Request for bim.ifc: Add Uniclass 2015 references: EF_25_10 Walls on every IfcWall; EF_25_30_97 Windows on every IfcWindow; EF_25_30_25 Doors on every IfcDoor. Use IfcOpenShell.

First a look at what the model holds.

```python
import ifcopenshell

model = ifcopenshell.open("bim.ifc")
print(model.schema)
print("classifications:", [c.Name for c in model.by_type("IfcClassification")])
for ifc_class in ("IfcDoor", "IfcRoof", "IfcStair", "IfcWall", "IfcWindow"):
    print(ifc_class, len(model.by_type(ifc_class)))
```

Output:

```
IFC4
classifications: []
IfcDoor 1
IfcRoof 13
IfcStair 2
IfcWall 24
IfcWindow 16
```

```python
import ifcopenshell
import ifcopenshell.api.classification

model = ifcopenshell.open("bim.ifc")

system = ifcopenshell.api.classification.add_classification(model, classification="Uniclass 2015")

codes = {
    "IfcWall": ("EF_25_10", "Walls"),
    "IfcWindow": ("EF_25_30_97", "Windows"),
    "IfcDoor": ("EF_25_30_25", "Doors"),
}
for ifc_class, (code, name) in codes.items():
    products = model.by_type(ifc_class)
    ifcopenshell.api.classification.add_reference(
        model, products=products, classification=system, identification=code, name=name
    )
    print(code, len(products))

model.write("bim_updated.ifc")
```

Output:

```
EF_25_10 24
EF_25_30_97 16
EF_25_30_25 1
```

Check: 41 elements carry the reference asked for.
